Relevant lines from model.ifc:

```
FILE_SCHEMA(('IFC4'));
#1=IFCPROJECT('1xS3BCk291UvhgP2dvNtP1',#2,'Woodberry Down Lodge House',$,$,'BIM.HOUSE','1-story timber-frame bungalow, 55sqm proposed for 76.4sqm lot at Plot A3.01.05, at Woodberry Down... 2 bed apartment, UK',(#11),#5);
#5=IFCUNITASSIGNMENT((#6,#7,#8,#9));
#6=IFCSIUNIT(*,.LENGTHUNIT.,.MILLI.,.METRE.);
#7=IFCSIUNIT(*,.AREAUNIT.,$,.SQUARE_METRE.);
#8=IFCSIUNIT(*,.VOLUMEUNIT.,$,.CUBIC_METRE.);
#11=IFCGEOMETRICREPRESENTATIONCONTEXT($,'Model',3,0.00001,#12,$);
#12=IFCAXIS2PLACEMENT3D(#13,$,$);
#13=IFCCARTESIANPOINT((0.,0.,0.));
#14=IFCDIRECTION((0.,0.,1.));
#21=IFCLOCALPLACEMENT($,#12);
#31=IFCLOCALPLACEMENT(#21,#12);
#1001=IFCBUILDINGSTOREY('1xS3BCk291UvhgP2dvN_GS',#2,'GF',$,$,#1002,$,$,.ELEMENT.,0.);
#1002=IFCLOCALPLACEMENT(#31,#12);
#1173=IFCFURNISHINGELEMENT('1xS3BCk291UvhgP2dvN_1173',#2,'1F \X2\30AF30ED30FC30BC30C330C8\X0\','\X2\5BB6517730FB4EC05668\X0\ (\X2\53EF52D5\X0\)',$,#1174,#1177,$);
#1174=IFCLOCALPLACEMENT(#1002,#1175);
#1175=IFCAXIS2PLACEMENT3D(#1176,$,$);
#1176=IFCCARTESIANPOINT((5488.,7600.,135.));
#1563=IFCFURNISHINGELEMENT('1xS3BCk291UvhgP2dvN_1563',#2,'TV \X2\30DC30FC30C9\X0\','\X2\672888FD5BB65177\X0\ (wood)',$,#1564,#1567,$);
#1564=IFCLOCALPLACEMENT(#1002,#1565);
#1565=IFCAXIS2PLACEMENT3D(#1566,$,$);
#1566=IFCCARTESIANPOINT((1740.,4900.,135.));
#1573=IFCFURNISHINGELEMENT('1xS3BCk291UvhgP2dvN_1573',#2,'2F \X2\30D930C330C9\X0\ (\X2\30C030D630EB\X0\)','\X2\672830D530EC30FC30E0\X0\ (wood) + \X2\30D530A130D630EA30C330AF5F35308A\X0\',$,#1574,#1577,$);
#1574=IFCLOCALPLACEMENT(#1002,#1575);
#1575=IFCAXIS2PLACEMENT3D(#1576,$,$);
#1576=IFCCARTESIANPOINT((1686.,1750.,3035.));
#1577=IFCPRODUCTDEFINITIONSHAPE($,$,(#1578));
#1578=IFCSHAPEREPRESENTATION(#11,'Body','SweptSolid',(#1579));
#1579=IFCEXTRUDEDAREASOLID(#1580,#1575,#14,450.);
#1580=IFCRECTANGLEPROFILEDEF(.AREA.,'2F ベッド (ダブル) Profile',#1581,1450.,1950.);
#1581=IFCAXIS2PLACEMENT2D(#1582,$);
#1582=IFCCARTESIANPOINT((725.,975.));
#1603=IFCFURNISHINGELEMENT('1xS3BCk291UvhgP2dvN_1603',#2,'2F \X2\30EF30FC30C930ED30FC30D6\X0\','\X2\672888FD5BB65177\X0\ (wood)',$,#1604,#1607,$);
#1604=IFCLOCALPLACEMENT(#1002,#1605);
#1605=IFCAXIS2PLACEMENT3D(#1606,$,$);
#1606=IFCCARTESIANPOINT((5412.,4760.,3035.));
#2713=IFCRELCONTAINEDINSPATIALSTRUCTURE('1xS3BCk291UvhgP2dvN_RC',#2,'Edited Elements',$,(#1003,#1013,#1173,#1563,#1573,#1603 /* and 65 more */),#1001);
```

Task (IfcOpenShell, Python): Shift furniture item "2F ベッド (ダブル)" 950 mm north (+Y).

```python
import ifcopenshell
import ifcopenshell.api.geometry
import ifcopenshell.util.placement
import ifcopenshell.util.unit

model = ifcopenshell.open("model.ifc")
unit_scale = ifcopenshell.util.unit.calculate_unit_scale(model)

item = model.by_id(1573)
matrix = ifcopenshell.util.placement.get_local_placement(item.ObjectPlacement)
matrix[1, 3] += 0.95 / unit_scale
ifcopenshell.api.geometry.edit_object_placement(model, product=item, matrix=matrix, is_si=False)

print(ifcopenshell.util.placement.get_local_placement(item.ObjectPlacement).round(3) + 0.0)

model.write("model_edited.ifc")
```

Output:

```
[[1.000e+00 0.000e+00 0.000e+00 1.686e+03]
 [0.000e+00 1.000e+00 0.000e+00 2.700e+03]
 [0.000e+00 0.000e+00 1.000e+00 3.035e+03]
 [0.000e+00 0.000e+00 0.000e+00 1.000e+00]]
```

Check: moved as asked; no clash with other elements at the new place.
